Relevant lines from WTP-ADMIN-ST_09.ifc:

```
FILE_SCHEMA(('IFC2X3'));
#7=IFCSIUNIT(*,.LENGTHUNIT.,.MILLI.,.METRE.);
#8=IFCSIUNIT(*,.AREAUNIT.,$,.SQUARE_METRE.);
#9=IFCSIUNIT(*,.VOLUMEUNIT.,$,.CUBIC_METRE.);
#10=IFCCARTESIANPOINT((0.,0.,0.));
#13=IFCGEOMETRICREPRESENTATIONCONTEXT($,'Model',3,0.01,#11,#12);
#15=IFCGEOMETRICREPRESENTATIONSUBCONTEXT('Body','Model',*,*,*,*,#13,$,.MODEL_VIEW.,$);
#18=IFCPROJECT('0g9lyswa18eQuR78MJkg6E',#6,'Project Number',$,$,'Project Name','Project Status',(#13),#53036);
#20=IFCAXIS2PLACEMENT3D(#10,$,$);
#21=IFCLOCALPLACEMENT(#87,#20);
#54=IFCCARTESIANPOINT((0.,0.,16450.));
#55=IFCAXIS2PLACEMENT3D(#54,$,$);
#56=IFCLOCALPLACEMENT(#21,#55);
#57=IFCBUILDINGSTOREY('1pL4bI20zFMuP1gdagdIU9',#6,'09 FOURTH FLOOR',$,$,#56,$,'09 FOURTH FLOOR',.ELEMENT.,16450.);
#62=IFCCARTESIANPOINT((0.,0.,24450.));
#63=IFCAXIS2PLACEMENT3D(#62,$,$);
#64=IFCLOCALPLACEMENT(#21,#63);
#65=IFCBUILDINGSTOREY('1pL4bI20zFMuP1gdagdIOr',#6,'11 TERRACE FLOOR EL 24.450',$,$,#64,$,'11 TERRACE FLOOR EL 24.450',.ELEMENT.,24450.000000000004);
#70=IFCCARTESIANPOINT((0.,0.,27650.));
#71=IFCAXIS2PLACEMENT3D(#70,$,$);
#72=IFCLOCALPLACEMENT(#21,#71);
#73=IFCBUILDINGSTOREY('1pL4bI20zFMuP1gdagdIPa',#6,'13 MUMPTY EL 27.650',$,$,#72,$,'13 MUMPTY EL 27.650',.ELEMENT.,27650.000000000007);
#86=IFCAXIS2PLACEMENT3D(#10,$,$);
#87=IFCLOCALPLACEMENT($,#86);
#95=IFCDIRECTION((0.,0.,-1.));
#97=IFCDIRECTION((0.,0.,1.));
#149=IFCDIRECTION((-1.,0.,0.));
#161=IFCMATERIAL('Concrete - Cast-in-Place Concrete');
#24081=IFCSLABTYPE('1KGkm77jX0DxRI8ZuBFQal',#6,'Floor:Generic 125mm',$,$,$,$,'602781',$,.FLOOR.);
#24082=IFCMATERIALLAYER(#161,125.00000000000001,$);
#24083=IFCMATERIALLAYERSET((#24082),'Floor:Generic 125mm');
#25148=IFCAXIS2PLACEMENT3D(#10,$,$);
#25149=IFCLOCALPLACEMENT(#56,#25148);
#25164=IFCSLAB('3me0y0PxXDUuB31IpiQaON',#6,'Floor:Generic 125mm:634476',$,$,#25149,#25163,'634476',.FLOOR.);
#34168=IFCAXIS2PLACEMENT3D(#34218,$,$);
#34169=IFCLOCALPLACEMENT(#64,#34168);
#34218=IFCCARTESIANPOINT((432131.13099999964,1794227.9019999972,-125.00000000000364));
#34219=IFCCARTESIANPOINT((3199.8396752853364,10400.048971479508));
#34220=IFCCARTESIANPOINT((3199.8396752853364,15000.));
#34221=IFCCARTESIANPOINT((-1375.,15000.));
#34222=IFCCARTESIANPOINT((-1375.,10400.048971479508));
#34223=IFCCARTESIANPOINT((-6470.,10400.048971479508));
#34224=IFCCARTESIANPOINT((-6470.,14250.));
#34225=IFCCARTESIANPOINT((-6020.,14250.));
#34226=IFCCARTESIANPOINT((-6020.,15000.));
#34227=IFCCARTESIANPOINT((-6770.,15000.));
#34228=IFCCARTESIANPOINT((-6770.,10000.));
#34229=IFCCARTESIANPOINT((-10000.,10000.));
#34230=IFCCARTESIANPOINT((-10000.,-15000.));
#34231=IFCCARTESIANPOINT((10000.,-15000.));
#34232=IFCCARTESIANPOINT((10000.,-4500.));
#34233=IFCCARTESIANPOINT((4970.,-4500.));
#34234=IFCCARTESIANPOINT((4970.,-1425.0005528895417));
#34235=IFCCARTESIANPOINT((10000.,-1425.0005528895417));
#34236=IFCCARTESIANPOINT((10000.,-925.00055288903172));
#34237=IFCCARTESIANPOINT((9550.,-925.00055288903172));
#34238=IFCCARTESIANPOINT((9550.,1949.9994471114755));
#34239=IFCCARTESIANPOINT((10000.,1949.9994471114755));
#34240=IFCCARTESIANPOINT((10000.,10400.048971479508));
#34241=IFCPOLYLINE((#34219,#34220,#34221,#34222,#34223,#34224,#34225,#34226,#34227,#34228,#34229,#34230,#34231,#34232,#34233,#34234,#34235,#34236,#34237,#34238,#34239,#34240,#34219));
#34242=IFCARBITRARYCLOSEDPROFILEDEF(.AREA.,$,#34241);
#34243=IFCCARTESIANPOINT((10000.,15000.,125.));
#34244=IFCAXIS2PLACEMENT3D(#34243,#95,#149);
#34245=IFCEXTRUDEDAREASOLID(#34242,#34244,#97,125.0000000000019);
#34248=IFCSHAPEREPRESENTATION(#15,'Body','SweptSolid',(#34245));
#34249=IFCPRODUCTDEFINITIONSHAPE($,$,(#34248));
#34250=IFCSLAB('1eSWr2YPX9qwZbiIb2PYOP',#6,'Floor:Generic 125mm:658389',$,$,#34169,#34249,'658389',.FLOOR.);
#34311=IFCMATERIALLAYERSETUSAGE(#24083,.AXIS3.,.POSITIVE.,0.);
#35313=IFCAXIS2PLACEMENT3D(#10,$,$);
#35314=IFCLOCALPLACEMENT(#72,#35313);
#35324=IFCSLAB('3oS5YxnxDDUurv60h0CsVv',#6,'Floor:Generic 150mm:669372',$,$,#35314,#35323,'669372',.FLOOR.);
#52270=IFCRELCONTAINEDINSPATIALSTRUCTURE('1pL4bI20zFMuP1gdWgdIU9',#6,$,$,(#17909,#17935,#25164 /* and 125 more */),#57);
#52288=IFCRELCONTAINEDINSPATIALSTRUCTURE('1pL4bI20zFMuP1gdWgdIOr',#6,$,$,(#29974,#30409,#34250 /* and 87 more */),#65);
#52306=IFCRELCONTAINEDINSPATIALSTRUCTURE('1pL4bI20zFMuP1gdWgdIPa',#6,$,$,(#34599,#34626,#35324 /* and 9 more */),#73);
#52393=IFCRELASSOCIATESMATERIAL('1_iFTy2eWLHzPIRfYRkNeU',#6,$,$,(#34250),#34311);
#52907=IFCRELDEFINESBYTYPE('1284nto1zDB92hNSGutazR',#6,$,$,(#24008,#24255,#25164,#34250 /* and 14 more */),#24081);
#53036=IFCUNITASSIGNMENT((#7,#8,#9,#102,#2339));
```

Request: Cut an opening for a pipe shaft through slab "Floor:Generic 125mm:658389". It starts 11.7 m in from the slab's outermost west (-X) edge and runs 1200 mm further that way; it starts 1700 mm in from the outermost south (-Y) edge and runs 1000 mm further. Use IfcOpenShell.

```python
import numpy as np
import ifcopenshell
import ifcopenshell.api.feature
import ifcopenshell.api.geometry
import ifcopenshell.api.root
import ifcopenshell.geom
import ifcopenshell.util.placement
import ifcopenshell.util.representation
import ifcopenshell.util.shape
import ifcopenshell.util.unit

model = ifcopenshell.open("WTP-ADMIN-ST_09.ifc")
unit_scale = ifcopenshell.util.unit.calculate_unit_scale(model)
settings = ifcopenshell.geom.settings()


def volume(element):
    """Net volume in cubic metres, openings subtracted."""
    shape = ifcopenshell.geom.create_shape(settings, element)
    return ifcopenshell.util.shape.get_volume(shape.geometry)


slab = model.by_guid("1eSWr2YPX9qwZbiIb2PYOP")
before = volume(slab)

# Extent in the slab's own axes, in metres. The edges named are its -X and -Y sides.
slab_shape = ifcopenshell.geom.create_shape(settings, slab)
vertices = ifcopenshell.util.shape.get_vertices(slab_shape.geometry)
x_min, y_min, bottom = vertices.min(axis=0)
top = vertices[:, 2].max()

opening = ifcopenshell.api.root.create_entity(model, ifc_class="IfcOpeningElement", name="Pipe shaft opening")
context = ifcopenshell.util.representation.get_context(model, "Model", "Body", "MODEL_VIEW")
width, depth = 1.2, 1
outline = [(0.0, 0.0), (width, 0.0), (width, depth), (0.0, depth), (0.0, 0.0)]
# Overshoot both faces by 50 mm so the cut is clean.
shape = ifcopenshell.api.geometry.add_slab_representation(
    model, context=context, depth=top - bottom + 0.1, polyline=outline
)
ifcopenshell.api.geometry.assign_representation(model, product=opening, representation=shape)

matrix = ifcopenshell.util.placement.get_local_placement(slab.ObjectPlacement)
matrix[:, 3] = matrix @ np.append(np.array([x_min + 11.7, y_min + 1.7, bottom - 0.05]) / unit_scale, 1.0)
ifcopenshell.api.geometry.edit_object_placement(model, product=opening, matrix=matrix, is_si=False)
ifcopenshell.api.feature.add_feature(model, feature=opening, element=slab)

after = volume(slab)

print(f"slab volume {before:.3f} -> {after:.3f} m3")

model.write("WTP-ADMIN-ST_09_edited.ifc")
```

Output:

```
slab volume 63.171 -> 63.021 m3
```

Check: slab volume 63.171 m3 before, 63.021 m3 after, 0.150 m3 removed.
